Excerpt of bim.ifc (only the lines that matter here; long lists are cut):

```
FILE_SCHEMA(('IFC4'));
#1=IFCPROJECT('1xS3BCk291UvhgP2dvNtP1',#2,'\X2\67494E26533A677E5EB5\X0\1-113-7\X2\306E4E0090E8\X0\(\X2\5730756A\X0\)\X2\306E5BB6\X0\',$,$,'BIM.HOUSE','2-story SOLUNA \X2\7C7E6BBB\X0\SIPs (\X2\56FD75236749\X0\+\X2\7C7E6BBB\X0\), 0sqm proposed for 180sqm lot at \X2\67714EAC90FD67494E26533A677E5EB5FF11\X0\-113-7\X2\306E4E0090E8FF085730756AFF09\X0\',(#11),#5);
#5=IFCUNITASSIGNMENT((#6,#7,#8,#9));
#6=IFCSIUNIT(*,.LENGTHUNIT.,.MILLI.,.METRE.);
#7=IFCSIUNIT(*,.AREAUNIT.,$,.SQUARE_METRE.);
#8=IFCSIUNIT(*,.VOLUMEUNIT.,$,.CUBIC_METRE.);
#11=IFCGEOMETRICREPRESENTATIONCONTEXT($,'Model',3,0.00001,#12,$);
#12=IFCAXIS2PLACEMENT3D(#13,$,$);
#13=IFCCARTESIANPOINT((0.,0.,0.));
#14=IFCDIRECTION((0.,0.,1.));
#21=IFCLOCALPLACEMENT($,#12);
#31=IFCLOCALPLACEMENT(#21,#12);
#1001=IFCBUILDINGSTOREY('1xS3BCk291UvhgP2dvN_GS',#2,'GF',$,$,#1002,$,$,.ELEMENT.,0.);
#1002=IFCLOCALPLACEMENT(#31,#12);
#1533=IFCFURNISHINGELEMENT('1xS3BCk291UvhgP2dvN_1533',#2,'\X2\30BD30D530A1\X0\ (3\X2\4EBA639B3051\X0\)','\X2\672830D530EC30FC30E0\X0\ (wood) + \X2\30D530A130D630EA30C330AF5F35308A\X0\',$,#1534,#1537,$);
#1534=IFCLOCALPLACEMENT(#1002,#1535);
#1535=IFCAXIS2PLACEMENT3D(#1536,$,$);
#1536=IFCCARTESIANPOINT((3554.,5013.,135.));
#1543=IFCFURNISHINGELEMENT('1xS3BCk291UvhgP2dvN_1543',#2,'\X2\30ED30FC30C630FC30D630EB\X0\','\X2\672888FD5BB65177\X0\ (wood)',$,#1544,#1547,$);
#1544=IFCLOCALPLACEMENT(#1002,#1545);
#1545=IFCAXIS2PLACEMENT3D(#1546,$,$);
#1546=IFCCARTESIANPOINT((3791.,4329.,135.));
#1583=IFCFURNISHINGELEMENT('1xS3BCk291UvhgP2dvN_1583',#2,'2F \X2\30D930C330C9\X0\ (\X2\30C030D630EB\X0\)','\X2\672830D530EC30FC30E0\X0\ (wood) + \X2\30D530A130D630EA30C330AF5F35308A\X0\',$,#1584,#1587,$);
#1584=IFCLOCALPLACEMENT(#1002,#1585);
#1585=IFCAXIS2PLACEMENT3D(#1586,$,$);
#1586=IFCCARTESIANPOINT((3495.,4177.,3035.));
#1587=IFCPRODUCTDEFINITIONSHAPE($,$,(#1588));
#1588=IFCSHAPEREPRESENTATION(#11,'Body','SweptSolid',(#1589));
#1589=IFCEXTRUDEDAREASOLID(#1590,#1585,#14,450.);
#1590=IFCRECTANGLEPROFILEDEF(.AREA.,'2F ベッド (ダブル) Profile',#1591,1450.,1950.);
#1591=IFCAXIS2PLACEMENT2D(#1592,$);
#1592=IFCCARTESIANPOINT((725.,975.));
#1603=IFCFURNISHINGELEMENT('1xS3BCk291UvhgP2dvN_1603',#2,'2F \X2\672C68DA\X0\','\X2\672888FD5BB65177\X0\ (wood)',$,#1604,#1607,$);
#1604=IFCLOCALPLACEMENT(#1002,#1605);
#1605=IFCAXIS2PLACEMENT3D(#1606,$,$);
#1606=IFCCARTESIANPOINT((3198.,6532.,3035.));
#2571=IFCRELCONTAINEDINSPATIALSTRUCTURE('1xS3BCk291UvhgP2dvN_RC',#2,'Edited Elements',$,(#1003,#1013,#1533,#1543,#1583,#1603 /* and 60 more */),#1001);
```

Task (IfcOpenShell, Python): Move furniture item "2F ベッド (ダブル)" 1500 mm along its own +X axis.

```python
import ifcopenshell
import ifcopenshell.api.geometry
import ifcopenshell.util.placement
import ifcopenshell.util.unit

model = ifcopenshell.open("bim.ifc")
unit_scale = ifcopenshell.util.unit.calculate_unit_scale(model)

item = model.by_guid("1xS3BCk291UvhgP2dvN_1583")
matrix = ifcopenshell.util.placement.get_local_placement(item.ObjectPlacement)
matrix[:3, 3] += matrix[:3, 0] * 1.5 / unit_scale
ifcopenshell.api.geometry.edit_object_placement(model, product=item, matrix=matrix, is_si=False)

print(ifcopenshell.util.placement.get_local_placement(item.ObjectPlacement).round(3) + 0.0)

model.write("bim_v2.ifc")
```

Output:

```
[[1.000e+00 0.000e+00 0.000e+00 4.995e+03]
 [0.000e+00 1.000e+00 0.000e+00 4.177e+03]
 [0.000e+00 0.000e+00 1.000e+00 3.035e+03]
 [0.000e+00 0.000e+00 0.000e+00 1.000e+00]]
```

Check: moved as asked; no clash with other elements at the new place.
